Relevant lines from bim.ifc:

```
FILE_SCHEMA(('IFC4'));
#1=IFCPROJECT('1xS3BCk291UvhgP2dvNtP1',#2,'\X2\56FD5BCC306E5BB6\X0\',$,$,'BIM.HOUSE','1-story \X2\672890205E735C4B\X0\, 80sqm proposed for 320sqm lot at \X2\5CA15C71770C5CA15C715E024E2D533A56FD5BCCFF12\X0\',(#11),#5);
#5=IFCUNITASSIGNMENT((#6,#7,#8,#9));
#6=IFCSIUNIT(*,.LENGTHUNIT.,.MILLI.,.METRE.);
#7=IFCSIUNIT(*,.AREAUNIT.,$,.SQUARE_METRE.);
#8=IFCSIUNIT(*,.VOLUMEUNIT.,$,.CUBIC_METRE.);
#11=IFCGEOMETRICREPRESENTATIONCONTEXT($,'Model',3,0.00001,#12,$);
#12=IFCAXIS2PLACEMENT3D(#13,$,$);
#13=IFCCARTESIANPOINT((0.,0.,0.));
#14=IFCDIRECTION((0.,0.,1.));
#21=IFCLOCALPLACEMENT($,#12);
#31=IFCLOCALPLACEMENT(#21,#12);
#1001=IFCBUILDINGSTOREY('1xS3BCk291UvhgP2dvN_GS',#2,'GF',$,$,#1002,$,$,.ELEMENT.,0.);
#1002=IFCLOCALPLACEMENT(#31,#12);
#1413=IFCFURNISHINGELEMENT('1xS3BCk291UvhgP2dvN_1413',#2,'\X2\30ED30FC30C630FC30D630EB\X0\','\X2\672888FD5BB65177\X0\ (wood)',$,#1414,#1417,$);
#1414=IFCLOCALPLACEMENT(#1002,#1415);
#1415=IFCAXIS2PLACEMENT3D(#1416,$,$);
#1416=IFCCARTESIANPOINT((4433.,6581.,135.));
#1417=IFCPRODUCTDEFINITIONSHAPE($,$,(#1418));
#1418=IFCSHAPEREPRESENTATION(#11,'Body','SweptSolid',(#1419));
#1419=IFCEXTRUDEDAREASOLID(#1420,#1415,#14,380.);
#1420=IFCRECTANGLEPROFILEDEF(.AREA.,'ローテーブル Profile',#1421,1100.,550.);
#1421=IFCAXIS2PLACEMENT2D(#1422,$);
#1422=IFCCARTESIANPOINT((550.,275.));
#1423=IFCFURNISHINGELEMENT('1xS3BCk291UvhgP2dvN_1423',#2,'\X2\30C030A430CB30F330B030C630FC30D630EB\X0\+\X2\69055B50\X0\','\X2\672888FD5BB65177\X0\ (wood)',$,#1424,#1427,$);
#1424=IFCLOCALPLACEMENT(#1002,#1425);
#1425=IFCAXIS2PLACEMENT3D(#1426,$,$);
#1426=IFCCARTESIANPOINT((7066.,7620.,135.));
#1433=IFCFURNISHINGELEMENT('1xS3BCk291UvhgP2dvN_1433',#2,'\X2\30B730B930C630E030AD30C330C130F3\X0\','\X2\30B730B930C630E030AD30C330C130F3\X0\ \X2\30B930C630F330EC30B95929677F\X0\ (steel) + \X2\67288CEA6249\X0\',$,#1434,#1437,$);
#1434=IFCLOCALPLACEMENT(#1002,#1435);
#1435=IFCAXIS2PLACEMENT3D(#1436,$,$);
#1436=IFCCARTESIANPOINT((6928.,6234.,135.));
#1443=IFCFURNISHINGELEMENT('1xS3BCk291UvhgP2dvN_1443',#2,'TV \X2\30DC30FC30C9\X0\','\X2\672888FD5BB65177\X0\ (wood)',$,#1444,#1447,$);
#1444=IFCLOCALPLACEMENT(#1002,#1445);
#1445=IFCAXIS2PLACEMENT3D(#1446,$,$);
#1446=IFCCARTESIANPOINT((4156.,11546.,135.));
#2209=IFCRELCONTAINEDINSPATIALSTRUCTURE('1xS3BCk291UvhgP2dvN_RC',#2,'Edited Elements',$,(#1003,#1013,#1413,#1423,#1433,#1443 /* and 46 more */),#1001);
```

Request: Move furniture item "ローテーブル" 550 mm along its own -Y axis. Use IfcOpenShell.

```python
import ifcopenshell
import ifcopenshell.api.geometry
import ifcopenshell.util.placement
import ifcopenshell.util.unit

model = ifcopenshell.open("bim.ifc")
unit_scale = ifcopenshell.util.unit.calculate_unit_scale(model)

item = model.by_id(1413)
matrix = ifcopenshell.util.placement.get_local_placement(item.ObjectPlacement)
matrix[:3, 3] -= matrix[:3, 1] * 0.55 / unit_scale
ifcopenshell.api.geometry.edit_object_placement(model, product=item, matrix=matrix, is_si=False)

print(ifcopenshell.util.placement.get_local_placement(item.ObjectPlacement).round(3) + 0.0)

model.write("bim_updated.ifc")
```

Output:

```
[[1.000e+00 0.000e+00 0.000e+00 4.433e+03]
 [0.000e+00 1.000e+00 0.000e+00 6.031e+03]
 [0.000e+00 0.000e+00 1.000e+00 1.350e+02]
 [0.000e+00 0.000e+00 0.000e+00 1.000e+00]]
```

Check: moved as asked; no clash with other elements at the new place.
